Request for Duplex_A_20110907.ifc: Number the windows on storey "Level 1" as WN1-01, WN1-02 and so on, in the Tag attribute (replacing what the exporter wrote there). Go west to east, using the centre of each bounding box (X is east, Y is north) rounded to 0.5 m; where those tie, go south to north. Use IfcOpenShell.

First a look at what the model holds.

```python
import ifcopenshell
import ifcopenshell.util.element
import ifcopenshell.util.placement

model = ifcopenshell.open("Duplex_A_20110907.ifc")
print(model.schema)
storey = next(s for s in model.by_type("IfcBuildingStorey") if s.Name == "Level 1")
windows = [e for e in ifcopenshell.util.element.get_decomposition(storey) if e.is_a("IfcWindow")]
for e in sorted(windows, key=lambda e: e.id()):
    origin = ifcopenshell.util.placement.get_local_placement(e.ObjectPlacement)[:3, 3]
    print(e.id(), e.Tag, e.Name, origin.round(2) + 0.0, sep=" | ")
```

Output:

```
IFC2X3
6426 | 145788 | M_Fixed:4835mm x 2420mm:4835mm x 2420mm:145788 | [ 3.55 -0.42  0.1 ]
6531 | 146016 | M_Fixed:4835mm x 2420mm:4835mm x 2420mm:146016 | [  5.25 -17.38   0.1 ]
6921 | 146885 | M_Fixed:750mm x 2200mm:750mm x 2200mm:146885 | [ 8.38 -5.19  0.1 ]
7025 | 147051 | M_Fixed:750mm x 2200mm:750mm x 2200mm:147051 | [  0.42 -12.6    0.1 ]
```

```python
import ifcopenshell
import ifcopenshell.geom
import ifcopenshell.util.element
import ifcopenshell.util.shape

model = ifcopenshell.open("Duplex_A_20110907.ifc")
settings = ifcopenshell.geom.settings()
settings.set("use-world-coords", True)


def centre(element):
    shape = ifcopenshell.geom.create_shape(settings, element)
    return ifcopenshell.util.shape.get_bbox_centroid(shape.geometry)


storey = next(s for s in model.by_type("IfcBuildingStorey") if s.Name == "Level 1")
windows = [e for e in ifcopenshell.util.element.get_decomposition(storey) if e.is_a("IfcWindow")]

# Insertion points can sit at a corner or the storey origin, so sort by the geometry (in metres).
centres = {e: centre(e) for e in windows}
windows.sort(key=lambda e: (round(centres[e][0] / 0.5), centres[e][1]))

for i, e in enumerate(windows, start=1):
    number = f"WN1-{i:02d}"
    e.Tag = number
    print(e.id(), number)

model.write("Duplex_A_20110907-out.ifc")
```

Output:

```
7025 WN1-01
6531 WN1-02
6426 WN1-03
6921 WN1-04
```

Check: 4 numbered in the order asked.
